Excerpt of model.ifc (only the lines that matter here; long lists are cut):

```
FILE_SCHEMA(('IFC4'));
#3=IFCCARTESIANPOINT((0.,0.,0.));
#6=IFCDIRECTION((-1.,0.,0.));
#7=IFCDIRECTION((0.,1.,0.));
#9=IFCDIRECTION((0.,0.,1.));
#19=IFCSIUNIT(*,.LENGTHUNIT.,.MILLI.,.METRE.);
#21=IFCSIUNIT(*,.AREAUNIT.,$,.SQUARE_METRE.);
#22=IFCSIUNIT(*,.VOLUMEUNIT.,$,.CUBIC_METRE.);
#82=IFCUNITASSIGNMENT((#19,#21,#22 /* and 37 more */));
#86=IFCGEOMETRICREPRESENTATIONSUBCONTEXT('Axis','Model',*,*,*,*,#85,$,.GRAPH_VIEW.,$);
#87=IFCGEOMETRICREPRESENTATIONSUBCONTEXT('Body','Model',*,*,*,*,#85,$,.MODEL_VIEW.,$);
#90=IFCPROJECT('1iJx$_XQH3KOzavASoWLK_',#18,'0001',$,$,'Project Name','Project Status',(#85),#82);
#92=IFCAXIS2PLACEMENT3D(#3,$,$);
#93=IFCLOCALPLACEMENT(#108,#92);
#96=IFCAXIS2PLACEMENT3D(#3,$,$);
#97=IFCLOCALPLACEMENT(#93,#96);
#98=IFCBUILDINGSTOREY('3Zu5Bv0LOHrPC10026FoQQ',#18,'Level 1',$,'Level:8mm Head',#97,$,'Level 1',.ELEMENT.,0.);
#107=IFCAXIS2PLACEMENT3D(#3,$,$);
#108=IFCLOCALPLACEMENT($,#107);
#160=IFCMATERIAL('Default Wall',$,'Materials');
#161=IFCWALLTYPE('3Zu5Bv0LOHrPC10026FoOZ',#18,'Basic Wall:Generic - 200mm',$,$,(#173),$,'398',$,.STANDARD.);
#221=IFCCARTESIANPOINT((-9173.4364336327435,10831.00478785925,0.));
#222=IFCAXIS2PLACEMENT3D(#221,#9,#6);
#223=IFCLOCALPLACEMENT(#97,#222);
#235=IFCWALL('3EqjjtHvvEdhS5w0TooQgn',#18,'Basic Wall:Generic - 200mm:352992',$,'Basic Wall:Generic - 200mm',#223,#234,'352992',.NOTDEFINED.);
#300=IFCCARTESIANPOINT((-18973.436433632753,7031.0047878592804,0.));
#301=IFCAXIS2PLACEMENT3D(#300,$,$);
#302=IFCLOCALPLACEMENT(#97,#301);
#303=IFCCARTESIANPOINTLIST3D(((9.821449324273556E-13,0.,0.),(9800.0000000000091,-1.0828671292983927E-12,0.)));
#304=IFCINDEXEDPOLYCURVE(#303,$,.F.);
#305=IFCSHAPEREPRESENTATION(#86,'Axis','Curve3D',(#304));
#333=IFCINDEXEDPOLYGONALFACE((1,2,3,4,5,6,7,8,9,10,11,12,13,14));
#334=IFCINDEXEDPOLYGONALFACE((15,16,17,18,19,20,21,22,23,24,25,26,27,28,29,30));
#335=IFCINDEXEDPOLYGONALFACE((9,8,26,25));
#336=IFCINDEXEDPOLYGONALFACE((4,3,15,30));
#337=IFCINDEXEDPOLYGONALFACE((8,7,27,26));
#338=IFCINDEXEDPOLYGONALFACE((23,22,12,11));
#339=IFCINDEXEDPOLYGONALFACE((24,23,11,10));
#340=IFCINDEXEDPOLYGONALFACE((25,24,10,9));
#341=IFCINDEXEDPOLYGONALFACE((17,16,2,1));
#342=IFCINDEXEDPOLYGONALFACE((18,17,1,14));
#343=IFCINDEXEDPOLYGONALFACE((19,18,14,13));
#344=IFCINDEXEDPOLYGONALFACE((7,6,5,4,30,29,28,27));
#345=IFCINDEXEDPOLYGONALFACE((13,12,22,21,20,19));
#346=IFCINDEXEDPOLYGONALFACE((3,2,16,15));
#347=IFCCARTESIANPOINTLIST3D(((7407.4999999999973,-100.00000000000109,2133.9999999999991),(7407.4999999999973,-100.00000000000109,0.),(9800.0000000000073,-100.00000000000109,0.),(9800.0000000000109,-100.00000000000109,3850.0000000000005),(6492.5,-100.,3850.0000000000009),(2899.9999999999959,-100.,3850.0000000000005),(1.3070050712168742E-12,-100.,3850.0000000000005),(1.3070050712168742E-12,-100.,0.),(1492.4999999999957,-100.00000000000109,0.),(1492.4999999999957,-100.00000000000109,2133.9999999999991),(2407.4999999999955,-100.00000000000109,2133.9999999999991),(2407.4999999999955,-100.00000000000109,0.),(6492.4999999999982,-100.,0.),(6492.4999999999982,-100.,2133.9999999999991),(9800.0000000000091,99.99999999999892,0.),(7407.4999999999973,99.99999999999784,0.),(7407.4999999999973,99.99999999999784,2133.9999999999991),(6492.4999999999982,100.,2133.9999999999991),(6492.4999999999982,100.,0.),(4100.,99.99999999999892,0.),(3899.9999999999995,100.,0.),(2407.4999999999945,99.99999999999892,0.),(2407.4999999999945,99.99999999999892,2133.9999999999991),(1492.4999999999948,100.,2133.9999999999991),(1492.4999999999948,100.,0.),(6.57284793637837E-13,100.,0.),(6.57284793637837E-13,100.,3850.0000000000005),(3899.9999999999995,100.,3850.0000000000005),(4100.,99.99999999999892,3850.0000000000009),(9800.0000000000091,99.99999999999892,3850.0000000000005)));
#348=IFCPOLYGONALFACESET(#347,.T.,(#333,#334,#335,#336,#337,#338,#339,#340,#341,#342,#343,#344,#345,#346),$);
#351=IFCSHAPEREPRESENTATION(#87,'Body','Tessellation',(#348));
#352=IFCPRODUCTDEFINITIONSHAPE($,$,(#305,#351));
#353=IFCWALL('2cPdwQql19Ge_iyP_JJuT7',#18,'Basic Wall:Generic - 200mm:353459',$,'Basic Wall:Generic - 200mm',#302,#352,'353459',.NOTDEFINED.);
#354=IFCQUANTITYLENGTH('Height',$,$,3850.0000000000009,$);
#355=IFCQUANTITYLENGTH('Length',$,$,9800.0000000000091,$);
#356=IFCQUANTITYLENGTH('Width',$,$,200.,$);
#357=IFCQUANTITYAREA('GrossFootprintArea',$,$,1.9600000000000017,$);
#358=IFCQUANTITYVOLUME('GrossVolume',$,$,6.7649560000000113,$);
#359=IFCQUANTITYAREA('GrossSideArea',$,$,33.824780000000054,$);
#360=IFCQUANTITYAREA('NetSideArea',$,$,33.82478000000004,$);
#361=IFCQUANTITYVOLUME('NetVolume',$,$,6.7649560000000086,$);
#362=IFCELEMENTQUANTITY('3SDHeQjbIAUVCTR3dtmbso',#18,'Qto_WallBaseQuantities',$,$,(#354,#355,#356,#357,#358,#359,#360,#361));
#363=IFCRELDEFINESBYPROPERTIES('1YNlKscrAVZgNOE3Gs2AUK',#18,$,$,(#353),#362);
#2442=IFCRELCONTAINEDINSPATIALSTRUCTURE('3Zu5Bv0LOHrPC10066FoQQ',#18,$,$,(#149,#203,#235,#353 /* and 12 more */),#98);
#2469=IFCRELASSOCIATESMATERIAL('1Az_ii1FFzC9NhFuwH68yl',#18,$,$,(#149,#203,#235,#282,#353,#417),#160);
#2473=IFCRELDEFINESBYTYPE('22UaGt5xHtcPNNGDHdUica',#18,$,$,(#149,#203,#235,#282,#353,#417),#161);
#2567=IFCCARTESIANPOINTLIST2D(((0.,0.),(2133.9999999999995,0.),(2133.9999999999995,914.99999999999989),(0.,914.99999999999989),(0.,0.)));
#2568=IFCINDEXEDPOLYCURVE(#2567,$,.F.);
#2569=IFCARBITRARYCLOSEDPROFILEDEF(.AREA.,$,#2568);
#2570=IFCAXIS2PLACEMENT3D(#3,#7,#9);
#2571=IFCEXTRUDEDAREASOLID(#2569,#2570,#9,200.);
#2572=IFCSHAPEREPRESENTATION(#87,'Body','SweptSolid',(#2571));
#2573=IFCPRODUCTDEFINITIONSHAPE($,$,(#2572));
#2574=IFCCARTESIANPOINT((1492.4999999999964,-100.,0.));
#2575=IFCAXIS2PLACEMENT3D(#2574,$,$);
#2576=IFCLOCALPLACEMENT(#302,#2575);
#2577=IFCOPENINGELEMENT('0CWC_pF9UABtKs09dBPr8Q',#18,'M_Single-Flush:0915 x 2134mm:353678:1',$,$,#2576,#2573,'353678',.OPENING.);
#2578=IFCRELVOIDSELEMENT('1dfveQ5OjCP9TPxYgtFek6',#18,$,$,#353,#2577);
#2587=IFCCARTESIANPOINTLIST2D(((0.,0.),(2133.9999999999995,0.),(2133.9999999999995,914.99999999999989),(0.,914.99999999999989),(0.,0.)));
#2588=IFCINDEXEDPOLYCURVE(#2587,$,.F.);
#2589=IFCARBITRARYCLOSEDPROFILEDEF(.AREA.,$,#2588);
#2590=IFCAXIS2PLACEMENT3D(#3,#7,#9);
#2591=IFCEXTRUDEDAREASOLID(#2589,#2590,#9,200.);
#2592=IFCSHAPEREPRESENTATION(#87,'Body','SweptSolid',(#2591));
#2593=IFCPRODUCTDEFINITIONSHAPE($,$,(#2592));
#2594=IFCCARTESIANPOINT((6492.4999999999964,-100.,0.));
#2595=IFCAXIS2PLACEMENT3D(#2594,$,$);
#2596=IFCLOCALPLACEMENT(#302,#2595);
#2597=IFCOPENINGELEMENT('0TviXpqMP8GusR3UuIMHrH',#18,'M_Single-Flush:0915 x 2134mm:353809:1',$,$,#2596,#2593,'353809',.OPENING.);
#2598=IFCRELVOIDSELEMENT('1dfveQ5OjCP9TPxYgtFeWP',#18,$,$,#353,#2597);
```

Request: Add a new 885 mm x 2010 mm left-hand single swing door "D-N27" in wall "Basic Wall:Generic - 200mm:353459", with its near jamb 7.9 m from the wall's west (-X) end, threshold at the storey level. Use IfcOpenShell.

```python
import numpy as np
import ifcopenshell
import ifcopenshell.api.feature
import ifcopenshell.api.geometry
import ifcopenshell.api.pset
import ifcopenshell.api.root
import ifcopenshell.api.spatial
import ifcopenshell.geom
import ifcopenshell.util.element
import ifcopenshell.util.placement
import ifcopenshell.util.representation
import ifcopenshell.util.shape
import ifcopenshell.util.unit

model = ifcopenshell.open("model.ifc")
unit_scale = ifcopenshell.util.unit.calculate_unit_scale(model)
area_scale = ifcopenshell.util.unit.calculate_unit_scale(model, "AREAUNIT")
volume_scale = ifcopenshell.util.unit.calculate_unit_scale(model, "VOLUMEUNIT")
settings = ifcopenshell.geom.settings()


def volume(element):
    """Net volume in cubic metres, openings subtracted."""
    shape = ifcopenshell.geom.create_shape(settings, element)
    return ifcopenshell.util.shape.get_volume(shape.geometry)


wall = model.by_id(353)
storey = ifcopenshell.util.element.get_container(wall, ifc_class="IfcBuildingStorey")
context = ifcopenshell.util.representation.get_context(model, "Model", "Body", "MODEL_VIEW")
before = volume(wall)

width, height, from_end, sill = 0.885, 2.01, 7.9, 0.0  # metres

# The wall runs along its own X axis, and the end named is its -X end.
wall_shape = ifcopenshell.geom.create_shape(settings, wall)
x, y, z = ifcopenshell.util.shape.get_vertices(wall_shape.geometry).T
start = x.min() + from_end
face, thickness = float(y.min()), float(y.max() - y.min())
wall_matrix = ifcopenshell.util.placement.get_local_placement(wall.ObjectPlacement)
level = ifcopenshell.util.placement.get_local_placement(storey.ObjectPlacement)[2, 3]


def in_wall(x, y):
    """Placement at x, y metres in the wall's axes, at sill height."""
    matrix = wall_matrix.copy()
    matrix[:, 3] = wall_matrix @ np.array([x / unit_scale, y / unit_scale, 0.0, 1.0])
    matrix[2, 3] = level + sill / unit_scale
    return matrix


# Opening: a box that overshoots both wall faces by 50 mm.
opening = ifcopenshell.api.root.create_entity(model, ifc_class="IfcOpeningElement", predefined_type="OPENING")
box = ifcopenshell.api.geometry.add_wall_representation(
    model, context=context, length=width, height=height, thickness=thickness + 0.1
)
ifcopenshell.api.geometry.assign_representation(model, product=opening, representation=box)
ifcopenshell.api.geometry.edit_object_placement(model, product=opening, matrix=in_wall(start, face - 0.05), is_si=False)
ifcopenshell.api.feature.add_feature(model, feature=opening, element=wall)

door = ifcopenshell.api.root.create_entity(model, ifc_class="IfcDoor", name="D-N27", predefined_type="DOOR")
door.OverallWidth, door.OverallHeight = width / unit_scale, height / unit_scale
door.OperationType = "SINGLE_SWING_LEFT"
body = ifcopenshell.api.geometry.add_door_representation(
    model,
    context=context,
    overall_width=door.OverallWidth,
    overall_height=door.OverallHeight,
    operation_type="SINGLE_SWING_LEFT",
    lining_properties={"LiningDepth": thickness / unit_scale, "ThresholdDepth": thickness / unit_scale},
)
ifcopenshell.api.geometry.assign_representation(model, product=door, representation=body)
ifcopenshell.api.spatial.assign_container(model, products=[door], relating_structure=storey)
ifcopenshell.api.feature.add_filling(model, opening=opening, element=door)

# The lining spans the wall, so the door starts at the wall face.
ifcopenshell.api.geometry.edit_object_placement(model, product=door, matrix=in_wall(start, face), is_si=False)

after = volume(wall)

# Update the wall's stored quantities.
qto = model.by_id(ifcopenshell.util.element.get_pset(wall, "Qto_WallBaseQuantities", should_inherit=False)["id"])
ifcopenshell.api.pset.edit_qto(model, qto=qto, properties={
    "NetSideArea": after / thickness / area_scale,
    "NetVolume": after / volume_scale,
})

print(f"wall volume {before:.3f} -> {after:.3f} m3")

model.write("model_updated.ifc")
```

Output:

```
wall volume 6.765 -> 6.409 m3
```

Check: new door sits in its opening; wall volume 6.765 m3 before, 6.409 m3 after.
